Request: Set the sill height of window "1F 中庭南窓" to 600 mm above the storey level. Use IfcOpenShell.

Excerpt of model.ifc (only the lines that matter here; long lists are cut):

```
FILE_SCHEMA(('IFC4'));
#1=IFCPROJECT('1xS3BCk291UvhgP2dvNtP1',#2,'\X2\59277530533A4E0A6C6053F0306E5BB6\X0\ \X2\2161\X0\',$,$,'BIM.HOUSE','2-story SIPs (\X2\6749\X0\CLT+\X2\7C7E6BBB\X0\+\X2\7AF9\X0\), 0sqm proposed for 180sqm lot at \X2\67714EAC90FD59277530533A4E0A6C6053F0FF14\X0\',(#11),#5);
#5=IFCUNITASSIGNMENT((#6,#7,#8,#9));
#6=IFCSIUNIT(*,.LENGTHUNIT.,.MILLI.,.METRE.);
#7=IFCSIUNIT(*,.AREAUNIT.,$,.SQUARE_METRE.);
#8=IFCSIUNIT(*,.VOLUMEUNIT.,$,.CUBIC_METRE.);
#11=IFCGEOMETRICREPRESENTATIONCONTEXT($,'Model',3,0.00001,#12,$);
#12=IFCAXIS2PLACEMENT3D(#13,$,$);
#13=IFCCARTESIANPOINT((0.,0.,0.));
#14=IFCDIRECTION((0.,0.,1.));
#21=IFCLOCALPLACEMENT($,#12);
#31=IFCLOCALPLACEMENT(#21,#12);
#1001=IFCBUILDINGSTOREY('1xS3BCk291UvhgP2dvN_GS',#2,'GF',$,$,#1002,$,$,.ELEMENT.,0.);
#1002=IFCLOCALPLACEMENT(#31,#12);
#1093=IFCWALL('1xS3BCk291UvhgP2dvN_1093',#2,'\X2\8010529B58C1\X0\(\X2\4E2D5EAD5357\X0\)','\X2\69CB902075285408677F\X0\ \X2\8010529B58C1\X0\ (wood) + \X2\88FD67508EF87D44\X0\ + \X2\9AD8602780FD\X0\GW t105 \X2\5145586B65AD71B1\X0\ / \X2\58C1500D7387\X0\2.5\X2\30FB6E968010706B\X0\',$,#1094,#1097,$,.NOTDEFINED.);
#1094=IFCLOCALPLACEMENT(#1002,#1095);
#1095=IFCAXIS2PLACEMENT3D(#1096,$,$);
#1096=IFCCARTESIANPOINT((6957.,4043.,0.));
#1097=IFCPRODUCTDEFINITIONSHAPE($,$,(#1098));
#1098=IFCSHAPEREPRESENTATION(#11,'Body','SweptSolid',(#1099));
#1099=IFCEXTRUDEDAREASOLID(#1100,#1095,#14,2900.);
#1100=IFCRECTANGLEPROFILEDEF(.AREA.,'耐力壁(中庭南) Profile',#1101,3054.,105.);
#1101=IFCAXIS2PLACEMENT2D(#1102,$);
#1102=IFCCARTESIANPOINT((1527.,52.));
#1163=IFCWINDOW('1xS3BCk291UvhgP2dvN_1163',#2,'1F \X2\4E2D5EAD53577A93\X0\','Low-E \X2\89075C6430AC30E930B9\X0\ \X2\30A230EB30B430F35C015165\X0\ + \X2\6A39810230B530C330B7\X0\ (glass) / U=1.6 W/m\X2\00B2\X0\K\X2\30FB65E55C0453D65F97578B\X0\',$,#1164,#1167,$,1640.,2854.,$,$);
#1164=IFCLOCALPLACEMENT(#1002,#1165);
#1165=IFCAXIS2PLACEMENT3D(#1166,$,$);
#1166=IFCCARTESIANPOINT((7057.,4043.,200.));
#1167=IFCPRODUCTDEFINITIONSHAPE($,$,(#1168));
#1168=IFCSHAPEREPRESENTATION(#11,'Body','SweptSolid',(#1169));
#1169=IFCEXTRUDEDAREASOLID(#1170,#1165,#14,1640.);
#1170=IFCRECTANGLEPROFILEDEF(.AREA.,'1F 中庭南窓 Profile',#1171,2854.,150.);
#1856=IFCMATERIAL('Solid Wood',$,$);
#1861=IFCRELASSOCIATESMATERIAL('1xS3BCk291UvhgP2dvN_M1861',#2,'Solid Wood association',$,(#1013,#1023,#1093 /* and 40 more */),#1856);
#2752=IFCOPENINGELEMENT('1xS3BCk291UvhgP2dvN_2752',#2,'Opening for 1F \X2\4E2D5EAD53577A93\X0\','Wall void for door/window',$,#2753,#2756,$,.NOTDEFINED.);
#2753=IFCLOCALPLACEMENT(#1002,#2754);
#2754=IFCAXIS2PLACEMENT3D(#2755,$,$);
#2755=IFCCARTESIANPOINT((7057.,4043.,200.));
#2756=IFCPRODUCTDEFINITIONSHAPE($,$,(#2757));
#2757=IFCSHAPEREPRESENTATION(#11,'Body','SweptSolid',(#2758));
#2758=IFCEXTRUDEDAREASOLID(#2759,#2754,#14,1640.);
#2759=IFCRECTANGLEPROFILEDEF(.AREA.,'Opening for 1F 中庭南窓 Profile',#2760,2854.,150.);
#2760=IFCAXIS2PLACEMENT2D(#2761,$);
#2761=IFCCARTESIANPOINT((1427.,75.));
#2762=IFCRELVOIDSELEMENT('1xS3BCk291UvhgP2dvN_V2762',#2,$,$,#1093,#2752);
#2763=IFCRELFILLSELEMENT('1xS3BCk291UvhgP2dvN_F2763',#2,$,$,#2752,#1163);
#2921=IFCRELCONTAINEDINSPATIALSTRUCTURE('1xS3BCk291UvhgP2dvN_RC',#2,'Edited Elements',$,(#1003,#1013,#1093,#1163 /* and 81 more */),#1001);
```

```python
import numpy as np
import ifcopenshell
import ifcopenshell.api.geometry
import ifcopenshell.geom
import ifcopenshell.util.element
import ifcopenshell.util.placement
import ifcopenshell.util.shape
import ifcopenshell.util.unit

model = ifcopenshell.open("model.ifc")
unit_scale = ifcopenshell.util.unit.calculate_unit_scale(model)

window = model.by_guid("1xS3BCk291UvhgP2dvN_1163")
opening = window.FillsVoids[0].RelatingOpeningElement
storey = ifcopenshell.util.element.get_container(window, ifc_class="IfcBuildingStorey")
level = ifcopenshell.util.placement.get_local_placement(storey.ObjectPlacement)[2, 3]

# The opening's origin need not be at the sill, so measure its lowest point.
shape = ifcopenshell.geom.create_shape(ifcopenshell.geom.settings(), opening)
bottom = ifcopenshell.util.shape.get_shape_bottom_elevation(shape, shape.geometry) / unit_scale
dz = level + 0.6 / unit_scale - bottom

shift = np.array([0.0, 0.0, dz])
# The window is not placed relative to its opening, so move both.
for product in (opening, window):
    matrix = ifcopenshell.util.placement.get_local_placement(product.ObjectPlacement)
    matrix[:3, 3] += shift
    ifcopenshell.api.geometry.edit_object_placement(model, product=product, matrix=matrix, is_si=False)

print(f"moved by {dz * unit_scale:+.3f} m")

model.write("model_v2.ifc")
```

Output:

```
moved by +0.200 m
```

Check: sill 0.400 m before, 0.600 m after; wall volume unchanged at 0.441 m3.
